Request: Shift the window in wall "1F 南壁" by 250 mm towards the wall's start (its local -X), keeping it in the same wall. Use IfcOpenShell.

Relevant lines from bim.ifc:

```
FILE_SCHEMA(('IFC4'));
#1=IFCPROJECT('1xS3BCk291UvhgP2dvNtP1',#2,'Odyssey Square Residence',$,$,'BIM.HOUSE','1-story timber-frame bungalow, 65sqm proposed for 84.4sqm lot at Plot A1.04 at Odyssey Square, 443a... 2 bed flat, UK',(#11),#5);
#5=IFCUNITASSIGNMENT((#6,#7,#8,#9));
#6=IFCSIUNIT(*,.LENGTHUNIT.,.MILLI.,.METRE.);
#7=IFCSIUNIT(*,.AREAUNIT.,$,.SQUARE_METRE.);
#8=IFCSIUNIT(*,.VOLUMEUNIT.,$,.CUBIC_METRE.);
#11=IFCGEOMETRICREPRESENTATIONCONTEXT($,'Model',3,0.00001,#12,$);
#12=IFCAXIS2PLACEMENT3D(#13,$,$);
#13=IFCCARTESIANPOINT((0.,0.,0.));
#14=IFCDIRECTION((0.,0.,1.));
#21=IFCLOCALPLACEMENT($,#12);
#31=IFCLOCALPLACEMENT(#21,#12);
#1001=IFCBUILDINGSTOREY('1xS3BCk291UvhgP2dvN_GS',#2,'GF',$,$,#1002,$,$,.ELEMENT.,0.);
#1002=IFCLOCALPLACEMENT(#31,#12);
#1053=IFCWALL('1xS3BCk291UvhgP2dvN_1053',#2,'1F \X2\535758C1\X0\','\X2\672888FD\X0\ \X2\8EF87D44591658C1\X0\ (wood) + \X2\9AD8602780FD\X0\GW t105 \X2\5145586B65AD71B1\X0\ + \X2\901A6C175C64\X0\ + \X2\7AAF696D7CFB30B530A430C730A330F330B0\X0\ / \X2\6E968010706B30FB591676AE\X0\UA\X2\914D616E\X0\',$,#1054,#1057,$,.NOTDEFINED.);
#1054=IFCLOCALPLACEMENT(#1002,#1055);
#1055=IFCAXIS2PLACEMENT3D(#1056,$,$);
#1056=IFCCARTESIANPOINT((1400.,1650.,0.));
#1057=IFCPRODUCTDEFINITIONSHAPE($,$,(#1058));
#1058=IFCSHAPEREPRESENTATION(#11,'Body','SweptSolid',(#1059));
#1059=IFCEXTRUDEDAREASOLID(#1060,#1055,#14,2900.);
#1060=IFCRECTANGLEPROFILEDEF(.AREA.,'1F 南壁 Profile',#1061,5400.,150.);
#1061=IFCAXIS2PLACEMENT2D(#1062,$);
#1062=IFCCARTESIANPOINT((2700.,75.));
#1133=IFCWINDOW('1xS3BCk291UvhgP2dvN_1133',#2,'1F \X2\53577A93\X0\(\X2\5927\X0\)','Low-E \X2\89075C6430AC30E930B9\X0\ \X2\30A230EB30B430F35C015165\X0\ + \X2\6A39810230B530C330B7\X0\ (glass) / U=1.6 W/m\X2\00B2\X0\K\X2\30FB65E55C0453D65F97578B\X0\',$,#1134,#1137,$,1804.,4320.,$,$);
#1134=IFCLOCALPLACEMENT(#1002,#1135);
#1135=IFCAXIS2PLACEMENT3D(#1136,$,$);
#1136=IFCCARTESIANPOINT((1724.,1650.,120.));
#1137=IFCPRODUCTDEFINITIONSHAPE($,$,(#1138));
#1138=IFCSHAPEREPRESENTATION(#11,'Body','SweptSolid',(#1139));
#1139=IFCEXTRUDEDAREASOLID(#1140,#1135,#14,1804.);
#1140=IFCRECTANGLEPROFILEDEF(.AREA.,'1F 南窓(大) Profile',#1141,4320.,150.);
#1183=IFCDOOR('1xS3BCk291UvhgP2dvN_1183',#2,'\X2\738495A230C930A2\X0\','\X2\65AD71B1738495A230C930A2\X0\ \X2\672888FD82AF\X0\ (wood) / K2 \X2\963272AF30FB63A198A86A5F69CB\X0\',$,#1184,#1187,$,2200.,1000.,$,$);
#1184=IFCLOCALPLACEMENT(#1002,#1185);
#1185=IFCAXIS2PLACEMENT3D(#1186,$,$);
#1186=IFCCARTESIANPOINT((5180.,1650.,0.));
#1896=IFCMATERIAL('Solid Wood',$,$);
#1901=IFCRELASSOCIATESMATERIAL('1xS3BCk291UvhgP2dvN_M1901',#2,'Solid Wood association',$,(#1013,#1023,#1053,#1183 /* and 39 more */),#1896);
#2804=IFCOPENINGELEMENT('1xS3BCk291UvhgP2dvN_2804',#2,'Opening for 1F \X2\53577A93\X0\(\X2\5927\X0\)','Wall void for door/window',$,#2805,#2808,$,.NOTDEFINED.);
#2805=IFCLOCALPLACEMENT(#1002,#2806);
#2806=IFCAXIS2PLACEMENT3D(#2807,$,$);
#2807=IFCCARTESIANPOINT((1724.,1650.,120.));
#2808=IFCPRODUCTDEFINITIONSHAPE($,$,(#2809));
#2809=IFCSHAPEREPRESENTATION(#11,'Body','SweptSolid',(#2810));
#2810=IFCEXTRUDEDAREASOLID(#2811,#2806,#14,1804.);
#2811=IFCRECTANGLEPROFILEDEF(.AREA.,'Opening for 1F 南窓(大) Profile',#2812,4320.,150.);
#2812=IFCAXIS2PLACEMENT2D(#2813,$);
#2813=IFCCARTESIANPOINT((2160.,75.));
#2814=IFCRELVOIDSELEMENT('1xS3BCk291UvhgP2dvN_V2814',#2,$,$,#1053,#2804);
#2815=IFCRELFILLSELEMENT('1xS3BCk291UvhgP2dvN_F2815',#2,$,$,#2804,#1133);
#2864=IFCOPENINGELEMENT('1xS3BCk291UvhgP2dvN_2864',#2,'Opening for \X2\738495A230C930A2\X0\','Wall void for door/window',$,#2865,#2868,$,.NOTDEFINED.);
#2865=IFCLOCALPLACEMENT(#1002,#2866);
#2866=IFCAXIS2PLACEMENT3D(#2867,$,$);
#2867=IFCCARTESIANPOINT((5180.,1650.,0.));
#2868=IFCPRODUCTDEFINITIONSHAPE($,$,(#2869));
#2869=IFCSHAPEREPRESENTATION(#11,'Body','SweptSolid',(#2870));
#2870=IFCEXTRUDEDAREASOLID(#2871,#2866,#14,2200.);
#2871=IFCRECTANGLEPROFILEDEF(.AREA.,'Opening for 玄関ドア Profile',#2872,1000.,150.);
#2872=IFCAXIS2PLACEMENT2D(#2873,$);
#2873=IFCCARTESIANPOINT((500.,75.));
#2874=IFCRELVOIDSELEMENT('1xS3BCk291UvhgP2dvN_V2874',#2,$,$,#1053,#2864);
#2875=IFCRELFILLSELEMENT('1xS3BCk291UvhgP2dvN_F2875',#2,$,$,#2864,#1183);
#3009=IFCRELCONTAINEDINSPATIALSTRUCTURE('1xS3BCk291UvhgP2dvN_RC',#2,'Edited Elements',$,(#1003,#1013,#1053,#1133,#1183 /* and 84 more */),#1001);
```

```python
import ifcopenshell
import ifcopenshell.api.geometry
import ifcopenshell.util.placement

model = ifcopenshell.open("bim.ifc")

window = model.by_guid("1xS3BCk291UvhgP2dvN_1133")
opening = window.FillsVoids[0].RelatingOpeningElement
wall = opening.VoidsElements[0].RelatingBuildingElement

wall_matrix = ifcopenshell.util.placement.get_local_placement(wall.ObjectPlacement)
shift = wall_matrix[:3, 0] * -250.0
before = ifcopenshell.util.placement.get_local_placement(window.ObjectPlacement)[:3, 3].copy()

# The window is not placed relative to its opening, so move both.
for product in (opening, window):
    matrix = ifcopenshell.util.placement.get_local_placement(product.ObjectPlacement)
    matrix[:3, 3] += shift
    ifcopenshell.api.geometry.edit_object_placement(model, product=product, matrix=matrix, is_si=False)

after = ifcopenshell.util.placement.get_local_placement(window.ObjectPlacement)[:3, 3]
print("window moved by", (after - before).round(3) + 0.0)

model.write("bim-out.ifc")
```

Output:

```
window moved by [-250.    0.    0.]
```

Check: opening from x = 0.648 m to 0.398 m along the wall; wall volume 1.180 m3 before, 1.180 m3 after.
